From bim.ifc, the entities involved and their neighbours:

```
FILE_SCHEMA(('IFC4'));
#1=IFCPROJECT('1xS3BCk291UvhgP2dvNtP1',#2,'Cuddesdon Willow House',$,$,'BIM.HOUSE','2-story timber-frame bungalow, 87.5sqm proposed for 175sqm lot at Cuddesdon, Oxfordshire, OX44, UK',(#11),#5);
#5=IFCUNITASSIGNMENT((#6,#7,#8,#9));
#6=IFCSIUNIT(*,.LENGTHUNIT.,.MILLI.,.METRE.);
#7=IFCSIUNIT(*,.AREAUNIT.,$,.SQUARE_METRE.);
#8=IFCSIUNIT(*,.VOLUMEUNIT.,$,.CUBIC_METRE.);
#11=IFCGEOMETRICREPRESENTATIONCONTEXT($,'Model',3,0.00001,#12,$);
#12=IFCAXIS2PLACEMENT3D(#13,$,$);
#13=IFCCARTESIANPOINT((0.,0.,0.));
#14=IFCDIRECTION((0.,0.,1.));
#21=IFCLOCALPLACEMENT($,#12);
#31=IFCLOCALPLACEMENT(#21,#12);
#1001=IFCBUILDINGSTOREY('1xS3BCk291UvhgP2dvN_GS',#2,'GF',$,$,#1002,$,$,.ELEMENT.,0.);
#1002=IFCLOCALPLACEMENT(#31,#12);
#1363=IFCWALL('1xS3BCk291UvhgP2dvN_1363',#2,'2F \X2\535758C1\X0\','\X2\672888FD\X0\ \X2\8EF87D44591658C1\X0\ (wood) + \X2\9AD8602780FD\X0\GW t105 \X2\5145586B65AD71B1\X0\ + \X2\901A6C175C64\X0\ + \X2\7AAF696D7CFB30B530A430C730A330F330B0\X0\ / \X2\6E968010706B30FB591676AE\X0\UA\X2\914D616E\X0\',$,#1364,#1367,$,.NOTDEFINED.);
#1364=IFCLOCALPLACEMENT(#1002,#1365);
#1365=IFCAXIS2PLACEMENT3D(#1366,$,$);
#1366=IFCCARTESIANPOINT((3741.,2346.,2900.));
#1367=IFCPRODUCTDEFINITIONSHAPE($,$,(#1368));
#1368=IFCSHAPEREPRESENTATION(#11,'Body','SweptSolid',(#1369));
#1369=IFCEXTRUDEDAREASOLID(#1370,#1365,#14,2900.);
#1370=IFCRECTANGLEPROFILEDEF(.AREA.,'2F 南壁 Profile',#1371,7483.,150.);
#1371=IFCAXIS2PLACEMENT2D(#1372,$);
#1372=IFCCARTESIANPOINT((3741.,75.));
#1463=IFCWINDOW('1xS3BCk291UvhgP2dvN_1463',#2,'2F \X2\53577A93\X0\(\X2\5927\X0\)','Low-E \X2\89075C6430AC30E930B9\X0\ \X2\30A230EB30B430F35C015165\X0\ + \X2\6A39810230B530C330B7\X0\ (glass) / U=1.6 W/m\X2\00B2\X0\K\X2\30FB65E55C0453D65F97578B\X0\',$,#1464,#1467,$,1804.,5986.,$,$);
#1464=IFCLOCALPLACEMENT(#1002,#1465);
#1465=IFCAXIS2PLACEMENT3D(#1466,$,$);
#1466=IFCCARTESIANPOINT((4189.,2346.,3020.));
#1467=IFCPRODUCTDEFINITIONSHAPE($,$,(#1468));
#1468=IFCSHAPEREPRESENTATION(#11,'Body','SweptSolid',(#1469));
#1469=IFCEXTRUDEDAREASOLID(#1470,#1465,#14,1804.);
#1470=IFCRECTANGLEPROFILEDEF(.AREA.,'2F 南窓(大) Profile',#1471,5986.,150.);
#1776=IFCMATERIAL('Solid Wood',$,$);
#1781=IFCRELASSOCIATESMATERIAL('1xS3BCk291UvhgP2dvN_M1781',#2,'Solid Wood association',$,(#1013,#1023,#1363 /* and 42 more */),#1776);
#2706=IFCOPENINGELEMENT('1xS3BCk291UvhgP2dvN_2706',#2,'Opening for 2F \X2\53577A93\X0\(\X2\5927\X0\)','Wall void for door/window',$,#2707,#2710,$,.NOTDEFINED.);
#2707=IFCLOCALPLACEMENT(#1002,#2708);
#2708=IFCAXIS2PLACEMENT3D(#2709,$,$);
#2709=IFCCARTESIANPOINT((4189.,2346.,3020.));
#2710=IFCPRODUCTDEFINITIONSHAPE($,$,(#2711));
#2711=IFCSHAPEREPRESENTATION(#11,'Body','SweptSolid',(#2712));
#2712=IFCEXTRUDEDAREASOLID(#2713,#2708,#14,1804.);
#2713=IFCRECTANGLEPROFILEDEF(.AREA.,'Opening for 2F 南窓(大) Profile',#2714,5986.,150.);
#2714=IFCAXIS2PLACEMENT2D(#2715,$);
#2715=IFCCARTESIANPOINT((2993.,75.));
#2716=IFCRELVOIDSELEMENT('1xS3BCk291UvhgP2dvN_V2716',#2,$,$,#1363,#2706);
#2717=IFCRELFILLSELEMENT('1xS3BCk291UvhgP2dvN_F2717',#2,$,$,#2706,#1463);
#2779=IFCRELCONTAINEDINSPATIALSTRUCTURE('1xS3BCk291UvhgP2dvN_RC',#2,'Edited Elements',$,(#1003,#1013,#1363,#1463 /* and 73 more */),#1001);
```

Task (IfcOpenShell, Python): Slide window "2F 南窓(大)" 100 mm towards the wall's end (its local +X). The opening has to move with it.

```python
import ifcopenshell
import ifcopenshell.api.geometry
import ifcopenshell.util.placement
import ifcopenshell.util.unit

model = ifcopenshell.open("bim.ifc")
unit_scale = ifcopenshell.util.unit.calculate_unit_scale(model)

window = model.by_id(1463)
opening = window.FillsVoids[0].RelatingOpeningElement
wall = opening.VoidsElements[0].RelatingBuildingElement

wall_matrix = ifcopenshell.util.placement.get_local_placement(wall.ObjectPlacement)
shift = wall_matrix[:3, 0] * 0.1 / unit_scale
before = ifcopenshell.util.placement.get_local_placement(window.ObjectPlacement)[:3, 3].copy()

# The window is not placed relative to its opening, so move both.
for product in (opening, window):
    matrix = ifcopenshell.util.placement.get_local_placement(product.ObjectPlacement)
    matrix[:3, 3] += shift
    ifcopenshell.api.geometry.edit_object_placement(model, product=product, matrix=matrix, is_si=False)

after = ifcopenshell.util.placement.get_local_placement(window.ObjectPlacement)[:3, 3]
print("window moved by", (after - before).round(3) + 0.0)

model.write("bim-out.ifc")
```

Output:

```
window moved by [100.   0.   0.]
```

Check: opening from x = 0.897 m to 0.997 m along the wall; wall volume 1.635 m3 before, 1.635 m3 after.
